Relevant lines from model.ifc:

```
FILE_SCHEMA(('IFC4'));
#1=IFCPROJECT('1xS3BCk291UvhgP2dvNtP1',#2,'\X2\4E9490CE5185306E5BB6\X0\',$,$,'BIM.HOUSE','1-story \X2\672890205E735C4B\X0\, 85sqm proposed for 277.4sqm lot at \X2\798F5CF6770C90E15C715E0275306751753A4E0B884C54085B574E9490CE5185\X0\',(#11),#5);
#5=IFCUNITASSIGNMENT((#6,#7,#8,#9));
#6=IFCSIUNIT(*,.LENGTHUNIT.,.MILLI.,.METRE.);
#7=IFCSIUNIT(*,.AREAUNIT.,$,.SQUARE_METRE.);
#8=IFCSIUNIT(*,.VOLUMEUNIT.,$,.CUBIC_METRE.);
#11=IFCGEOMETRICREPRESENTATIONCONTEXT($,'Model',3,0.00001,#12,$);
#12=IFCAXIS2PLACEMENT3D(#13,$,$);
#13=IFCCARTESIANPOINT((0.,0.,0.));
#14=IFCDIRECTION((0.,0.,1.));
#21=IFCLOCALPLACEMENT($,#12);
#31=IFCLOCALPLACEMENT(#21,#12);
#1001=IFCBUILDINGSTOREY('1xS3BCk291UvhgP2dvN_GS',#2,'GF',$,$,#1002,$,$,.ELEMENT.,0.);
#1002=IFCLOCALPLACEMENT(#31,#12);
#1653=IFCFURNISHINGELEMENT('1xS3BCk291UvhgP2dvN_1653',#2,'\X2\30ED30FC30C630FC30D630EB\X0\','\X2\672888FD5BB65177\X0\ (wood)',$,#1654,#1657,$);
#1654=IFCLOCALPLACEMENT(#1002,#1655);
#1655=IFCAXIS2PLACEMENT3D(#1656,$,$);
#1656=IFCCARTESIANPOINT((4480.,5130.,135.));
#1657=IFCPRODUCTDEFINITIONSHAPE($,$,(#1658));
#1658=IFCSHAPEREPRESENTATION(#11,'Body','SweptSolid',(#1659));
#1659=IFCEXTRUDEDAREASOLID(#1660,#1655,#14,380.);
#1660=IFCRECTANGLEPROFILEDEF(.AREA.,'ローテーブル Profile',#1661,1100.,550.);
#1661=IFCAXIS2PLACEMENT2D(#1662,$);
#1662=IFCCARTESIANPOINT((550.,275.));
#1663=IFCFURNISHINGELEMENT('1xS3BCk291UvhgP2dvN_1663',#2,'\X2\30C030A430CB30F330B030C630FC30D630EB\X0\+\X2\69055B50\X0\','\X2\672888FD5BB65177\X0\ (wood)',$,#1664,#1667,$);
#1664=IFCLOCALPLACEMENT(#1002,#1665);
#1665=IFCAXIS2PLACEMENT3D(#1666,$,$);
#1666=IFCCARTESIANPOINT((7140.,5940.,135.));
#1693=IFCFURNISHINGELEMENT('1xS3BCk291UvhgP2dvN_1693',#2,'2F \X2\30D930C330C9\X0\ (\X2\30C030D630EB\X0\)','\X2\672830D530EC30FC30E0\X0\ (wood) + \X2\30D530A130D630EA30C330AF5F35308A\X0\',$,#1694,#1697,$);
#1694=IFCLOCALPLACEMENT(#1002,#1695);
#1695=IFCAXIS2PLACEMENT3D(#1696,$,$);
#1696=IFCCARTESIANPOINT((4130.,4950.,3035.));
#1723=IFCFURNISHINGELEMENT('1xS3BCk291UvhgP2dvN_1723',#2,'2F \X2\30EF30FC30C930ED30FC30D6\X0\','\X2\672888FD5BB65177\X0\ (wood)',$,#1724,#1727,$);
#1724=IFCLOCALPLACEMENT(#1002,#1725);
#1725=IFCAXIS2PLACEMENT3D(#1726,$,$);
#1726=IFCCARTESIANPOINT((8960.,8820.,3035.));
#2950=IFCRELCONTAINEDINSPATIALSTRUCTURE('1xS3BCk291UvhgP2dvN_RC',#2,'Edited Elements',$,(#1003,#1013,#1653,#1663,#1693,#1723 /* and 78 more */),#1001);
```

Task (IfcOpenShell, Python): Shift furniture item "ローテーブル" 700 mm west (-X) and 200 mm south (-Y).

```python
import ifcopenshell
import ifcopenshell.api.geometry
import ifcopenshell.util.placement

model = ifcopenshell.open("model.ifc")

item = model.by_guid("1xS3BCk291UvhgP2dvN_1653")
matrix = ifcopenshell.util.placement.get_local_placement(item.ObjectPlacement)
matrix[0, 3] -= 700.0
matrix[1, 3] -= 200.0
ifcopenshell.api.geometry.edit_object_placement(model, product=item, matrix=matrix, is_si=False)

print(ifcopenshell.util.placement.get_local_placement(item.ObjectPlacement).round(3) + 0.0)

model.write("model_edited.ifc")
```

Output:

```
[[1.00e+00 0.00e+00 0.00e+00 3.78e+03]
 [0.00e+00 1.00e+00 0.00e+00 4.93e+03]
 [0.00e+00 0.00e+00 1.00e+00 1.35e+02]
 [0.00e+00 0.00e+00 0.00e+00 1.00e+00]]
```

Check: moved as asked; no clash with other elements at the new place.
